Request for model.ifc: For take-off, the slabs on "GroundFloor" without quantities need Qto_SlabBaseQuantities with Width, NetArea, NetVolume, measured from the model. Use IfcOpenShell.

First a look at what the model holds.

```python
import ifcopenshell
import ifcopenshell.util.element
import ifcopenshell.util.unit

model = ifcopenshell.open("model.ifc")
print(model.schema)
for unit_type in ("LENGTHUNIT", "AREAUNIT", "VOLUMEUNIT"):
    print(unit_type, ifcopenshell.util.unit.calculate_unit_scale(model, unit_type))
storey = next(s for s in model.by_type("IfcBuildingStorey") if s.Name == "GroundFloor")
slabs = [e for e in ifcopenshell.util.element.get_decomposition(storey) if e.is_a("IfcSlab")]
for e in sorted(slabs, key=lambda e: e.id()):
    print(e.id(), e.is_a(), e.Name, list(ifcopenshell.util.element.get_psets(e, qtos_only=True)), sep=" | ")
```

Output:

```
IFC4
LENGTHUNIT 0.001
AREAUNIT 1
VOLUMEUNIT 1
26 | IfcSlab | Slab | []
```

```python
import ifcopenshell
import ifcopenshell.api.pset
import ifcopenshell.geom
import ifcopenshell.util.element
import ifcopenshell.util.shape
import ifcopenshell.util.unit

model = ifcopenshell.open("model.ifc")
unit_scale = ifcopenshell.util.unit.calculate_unit_scale(model)
area_scale = ifcopenshell.util.unit.calculate_unit_scale(model, "AREAUNIT")
volume_scale = ifcopenshell.util.unit.calculate_unit_scale(model, "VOLUMEUNIT")
settings = ifcopenshell.geom.settings()

storey = next(s for s in model.by_type("IfcBuildingStorey") if s.Name == "GroundFloor")
slabs = [e for e in ifcopenshell.util.element.get_decomposition(storey) if e.is_a("IfcSlab")]

for e in sorted(slabs, key=lambda e: e.id()):
    if ifcopenshell.util.element.get_psets(e, qtos_only=True, should_inherit=False):
        continue
    # Geometry comes back in metres, in the element's own axes.
    shape = ifcopenshell.geom.create_shape(settings, e)
    values = {
        "Width": ifcopenshell.util.shape.get_z(shape.geometry) / unit_scale,
        "NetArea": ifcopenshell.util.shape.get_footprint_area(shape.geometry) / area_scale,
        "NetVolume": ifcopenshell.util.shape.get_volume(shape.geometry) / volume_scale,
    }
    qto = ifcopenshell.api.pset.add_qto(model, product=e, name="Qto_SlabBaseQuantities")
    ifcopenshell.api.pset.edit_qto(model, qto=qto, properties=values)
    print(e.id(), {k: round(v, 3) for k, v in values.items()})

model.write("model_rev.ifc")
```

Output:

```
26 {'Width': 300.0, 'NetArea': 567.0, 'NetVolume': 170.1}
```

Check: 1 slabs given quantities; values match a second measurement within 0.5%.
